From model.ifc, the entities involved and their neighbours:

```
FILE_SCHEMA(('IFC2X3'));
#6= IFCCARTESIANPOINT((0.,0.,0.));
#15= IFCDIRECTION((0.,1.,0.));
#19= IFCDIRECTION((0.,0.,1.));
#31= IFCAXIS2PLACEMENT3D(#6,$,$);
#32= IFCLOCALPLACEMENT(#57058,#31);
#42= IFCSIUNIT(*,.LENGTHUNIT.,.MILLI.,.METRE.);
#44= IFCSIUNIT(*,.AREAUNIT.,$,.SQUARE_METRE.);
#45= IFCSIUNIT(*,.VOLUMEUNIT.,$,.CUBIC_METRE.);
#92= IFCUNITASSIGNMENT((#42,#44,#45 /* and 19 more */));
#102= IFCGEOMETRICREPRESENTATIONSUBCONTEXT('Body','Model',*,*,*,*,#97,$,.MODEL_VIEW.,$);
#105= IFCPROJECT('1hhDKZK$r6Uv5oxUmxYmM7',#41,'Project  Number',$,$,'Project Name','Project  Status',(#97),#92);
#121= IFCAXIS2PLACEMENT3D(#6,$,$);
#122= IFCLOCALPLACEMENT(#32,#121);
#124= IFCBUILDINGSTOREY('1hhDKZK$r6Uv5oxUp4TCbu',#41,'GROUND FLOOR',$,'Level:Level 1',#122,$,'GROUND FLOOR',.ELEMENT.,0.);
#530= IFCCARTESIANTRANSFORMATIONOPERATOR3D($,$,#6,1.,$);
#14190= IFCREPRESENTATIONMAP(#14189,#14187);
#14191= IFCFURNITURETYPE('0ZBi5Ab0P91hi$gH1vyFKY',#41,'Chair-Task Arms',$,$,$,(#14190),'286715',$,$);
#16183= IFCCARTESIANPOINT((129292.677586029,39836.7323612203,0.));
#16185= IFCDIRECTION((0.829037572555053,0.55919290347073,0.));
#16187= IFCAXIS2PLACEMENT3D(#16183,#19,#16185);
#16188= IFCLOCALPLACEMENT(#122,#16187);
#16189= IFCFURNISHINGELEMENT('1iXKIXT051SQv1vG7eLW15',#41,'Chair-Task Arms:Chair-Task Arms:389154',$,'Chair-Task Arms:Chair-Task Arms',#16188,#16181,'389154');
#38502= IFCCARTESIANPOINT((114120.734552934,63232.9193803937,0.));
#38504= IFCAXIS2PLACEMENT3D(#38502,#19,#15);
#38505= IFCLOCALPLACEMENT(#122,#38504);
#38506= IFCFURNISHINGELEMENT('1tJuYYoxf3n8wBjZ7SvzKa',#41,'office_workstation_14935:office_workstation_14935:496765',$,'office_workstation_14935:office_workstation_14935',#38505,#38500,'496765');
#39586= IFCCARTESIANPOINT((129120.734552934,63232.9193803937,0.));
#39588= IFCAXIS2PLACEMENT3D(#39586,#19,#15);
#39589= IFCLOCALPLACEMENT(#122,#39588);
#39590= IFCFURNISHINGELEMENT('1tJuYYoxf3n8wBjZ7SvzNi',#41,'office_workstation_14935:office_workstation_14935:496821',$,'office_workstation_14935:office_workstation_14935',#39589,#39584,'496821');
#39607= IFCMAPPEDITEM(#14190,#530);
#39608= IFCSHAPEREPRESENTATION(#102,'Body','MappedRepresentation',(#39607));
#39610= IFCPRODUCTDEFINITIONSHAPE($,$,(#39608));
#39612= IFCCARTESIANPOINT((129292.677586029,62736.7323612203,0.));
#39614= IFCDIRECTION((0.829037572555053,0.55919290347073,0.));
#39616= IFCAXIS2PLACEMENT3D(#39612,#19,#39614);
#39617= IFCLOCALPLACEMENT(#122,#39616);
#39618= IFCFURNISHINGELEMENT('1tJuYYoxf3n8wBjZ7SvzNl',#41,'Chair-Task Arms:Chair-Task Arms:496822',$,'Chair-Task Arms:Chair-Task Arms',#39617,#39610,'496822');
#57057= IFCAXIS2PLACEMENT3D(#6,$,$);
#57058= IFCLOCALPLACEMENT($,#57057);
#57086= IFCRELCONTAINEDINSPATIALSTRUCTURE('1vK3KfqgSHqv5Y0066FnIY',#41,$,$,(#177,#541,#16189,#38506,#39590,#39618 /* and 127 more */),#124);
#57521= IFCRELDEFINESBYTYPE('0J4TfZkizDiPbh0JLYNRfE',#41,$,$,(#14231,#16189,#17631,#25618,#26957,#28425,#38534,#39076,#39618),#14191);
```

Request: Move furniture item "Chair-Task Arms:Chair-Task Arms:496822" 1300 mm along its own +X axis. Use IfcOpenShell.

```python
import ifcopenshell
import ifcopenshell.api.geometry
import ifcopenshell.util.placement
import ifcopenshell.util.unit

model = ifcopenshell.open("model.ifc")
unit_scale = ifcopenshell.util.unit.calculate_unit_scale(model)

item = model.by_id(39618)
matrix = ifcopenshell.util.placement.get_local_placement(item.ObjectPlacement)
matrix[:3, 3] += matrix[:3, 0] * 1.3 / unit_scale
ifcopenshell.api.geometry.edit_object_placement(model, product=item, matrix=matrix, is_si=False)

print(ifcopenshell.util.placement.get_local_placement(item.ObjectPlacement).round(3) + 0.0)

model.write("model_v2.ifc")
```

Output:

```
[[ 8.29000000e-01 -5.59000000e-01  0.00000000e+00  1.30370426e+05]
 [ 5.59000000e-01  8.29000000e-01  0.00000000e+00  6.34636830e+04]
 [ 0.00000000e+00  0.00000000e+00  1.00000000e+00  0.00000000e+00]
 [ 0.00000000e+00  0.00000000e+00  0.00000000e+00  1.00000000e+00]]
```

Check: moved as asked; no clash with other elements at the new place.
